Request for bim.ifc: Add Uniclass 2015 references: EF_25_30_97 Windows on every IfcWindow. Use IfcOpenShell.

First a look at what the model holds.

```python
import ifcopenshell

model = ifcopenshell.open("bim.ifc")
print(model.schema)
print("classifications:", [c.Name for c in model.by_type("IfcClassification")])
for ifc_class in ("IfcDoor", "IfcRoof", "IfcStair", "IfcWall", "IfcWindow"):
    print(ifc_class, len(model.by_type(ifc_class)))
```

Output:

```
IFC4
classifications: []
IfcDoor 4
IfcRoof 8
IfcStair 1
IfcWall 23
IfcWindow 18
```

```python
import ifcopenshell
import ifcopenshell.api.classification

model = ifcopenshell.open("bim.ifc")

system = ifcopenshell.api.classification.add_classification(model, classification="Uniclass 2015")

codes = {
    "IfcWindow": ("EF_25_30_97", "Windows"),
}
for ifc_class, (code, name) in codes.items():
    products = model.by_type(ifc_class)
    ifcopenshell.api.classification.add_reference(
        model, products=products, classification=system, identification=code, name=name
    )
    print(code, len(products))

model.write("bim_updated.ifc")
```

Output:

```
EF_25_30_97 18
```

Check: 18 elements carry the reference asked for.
